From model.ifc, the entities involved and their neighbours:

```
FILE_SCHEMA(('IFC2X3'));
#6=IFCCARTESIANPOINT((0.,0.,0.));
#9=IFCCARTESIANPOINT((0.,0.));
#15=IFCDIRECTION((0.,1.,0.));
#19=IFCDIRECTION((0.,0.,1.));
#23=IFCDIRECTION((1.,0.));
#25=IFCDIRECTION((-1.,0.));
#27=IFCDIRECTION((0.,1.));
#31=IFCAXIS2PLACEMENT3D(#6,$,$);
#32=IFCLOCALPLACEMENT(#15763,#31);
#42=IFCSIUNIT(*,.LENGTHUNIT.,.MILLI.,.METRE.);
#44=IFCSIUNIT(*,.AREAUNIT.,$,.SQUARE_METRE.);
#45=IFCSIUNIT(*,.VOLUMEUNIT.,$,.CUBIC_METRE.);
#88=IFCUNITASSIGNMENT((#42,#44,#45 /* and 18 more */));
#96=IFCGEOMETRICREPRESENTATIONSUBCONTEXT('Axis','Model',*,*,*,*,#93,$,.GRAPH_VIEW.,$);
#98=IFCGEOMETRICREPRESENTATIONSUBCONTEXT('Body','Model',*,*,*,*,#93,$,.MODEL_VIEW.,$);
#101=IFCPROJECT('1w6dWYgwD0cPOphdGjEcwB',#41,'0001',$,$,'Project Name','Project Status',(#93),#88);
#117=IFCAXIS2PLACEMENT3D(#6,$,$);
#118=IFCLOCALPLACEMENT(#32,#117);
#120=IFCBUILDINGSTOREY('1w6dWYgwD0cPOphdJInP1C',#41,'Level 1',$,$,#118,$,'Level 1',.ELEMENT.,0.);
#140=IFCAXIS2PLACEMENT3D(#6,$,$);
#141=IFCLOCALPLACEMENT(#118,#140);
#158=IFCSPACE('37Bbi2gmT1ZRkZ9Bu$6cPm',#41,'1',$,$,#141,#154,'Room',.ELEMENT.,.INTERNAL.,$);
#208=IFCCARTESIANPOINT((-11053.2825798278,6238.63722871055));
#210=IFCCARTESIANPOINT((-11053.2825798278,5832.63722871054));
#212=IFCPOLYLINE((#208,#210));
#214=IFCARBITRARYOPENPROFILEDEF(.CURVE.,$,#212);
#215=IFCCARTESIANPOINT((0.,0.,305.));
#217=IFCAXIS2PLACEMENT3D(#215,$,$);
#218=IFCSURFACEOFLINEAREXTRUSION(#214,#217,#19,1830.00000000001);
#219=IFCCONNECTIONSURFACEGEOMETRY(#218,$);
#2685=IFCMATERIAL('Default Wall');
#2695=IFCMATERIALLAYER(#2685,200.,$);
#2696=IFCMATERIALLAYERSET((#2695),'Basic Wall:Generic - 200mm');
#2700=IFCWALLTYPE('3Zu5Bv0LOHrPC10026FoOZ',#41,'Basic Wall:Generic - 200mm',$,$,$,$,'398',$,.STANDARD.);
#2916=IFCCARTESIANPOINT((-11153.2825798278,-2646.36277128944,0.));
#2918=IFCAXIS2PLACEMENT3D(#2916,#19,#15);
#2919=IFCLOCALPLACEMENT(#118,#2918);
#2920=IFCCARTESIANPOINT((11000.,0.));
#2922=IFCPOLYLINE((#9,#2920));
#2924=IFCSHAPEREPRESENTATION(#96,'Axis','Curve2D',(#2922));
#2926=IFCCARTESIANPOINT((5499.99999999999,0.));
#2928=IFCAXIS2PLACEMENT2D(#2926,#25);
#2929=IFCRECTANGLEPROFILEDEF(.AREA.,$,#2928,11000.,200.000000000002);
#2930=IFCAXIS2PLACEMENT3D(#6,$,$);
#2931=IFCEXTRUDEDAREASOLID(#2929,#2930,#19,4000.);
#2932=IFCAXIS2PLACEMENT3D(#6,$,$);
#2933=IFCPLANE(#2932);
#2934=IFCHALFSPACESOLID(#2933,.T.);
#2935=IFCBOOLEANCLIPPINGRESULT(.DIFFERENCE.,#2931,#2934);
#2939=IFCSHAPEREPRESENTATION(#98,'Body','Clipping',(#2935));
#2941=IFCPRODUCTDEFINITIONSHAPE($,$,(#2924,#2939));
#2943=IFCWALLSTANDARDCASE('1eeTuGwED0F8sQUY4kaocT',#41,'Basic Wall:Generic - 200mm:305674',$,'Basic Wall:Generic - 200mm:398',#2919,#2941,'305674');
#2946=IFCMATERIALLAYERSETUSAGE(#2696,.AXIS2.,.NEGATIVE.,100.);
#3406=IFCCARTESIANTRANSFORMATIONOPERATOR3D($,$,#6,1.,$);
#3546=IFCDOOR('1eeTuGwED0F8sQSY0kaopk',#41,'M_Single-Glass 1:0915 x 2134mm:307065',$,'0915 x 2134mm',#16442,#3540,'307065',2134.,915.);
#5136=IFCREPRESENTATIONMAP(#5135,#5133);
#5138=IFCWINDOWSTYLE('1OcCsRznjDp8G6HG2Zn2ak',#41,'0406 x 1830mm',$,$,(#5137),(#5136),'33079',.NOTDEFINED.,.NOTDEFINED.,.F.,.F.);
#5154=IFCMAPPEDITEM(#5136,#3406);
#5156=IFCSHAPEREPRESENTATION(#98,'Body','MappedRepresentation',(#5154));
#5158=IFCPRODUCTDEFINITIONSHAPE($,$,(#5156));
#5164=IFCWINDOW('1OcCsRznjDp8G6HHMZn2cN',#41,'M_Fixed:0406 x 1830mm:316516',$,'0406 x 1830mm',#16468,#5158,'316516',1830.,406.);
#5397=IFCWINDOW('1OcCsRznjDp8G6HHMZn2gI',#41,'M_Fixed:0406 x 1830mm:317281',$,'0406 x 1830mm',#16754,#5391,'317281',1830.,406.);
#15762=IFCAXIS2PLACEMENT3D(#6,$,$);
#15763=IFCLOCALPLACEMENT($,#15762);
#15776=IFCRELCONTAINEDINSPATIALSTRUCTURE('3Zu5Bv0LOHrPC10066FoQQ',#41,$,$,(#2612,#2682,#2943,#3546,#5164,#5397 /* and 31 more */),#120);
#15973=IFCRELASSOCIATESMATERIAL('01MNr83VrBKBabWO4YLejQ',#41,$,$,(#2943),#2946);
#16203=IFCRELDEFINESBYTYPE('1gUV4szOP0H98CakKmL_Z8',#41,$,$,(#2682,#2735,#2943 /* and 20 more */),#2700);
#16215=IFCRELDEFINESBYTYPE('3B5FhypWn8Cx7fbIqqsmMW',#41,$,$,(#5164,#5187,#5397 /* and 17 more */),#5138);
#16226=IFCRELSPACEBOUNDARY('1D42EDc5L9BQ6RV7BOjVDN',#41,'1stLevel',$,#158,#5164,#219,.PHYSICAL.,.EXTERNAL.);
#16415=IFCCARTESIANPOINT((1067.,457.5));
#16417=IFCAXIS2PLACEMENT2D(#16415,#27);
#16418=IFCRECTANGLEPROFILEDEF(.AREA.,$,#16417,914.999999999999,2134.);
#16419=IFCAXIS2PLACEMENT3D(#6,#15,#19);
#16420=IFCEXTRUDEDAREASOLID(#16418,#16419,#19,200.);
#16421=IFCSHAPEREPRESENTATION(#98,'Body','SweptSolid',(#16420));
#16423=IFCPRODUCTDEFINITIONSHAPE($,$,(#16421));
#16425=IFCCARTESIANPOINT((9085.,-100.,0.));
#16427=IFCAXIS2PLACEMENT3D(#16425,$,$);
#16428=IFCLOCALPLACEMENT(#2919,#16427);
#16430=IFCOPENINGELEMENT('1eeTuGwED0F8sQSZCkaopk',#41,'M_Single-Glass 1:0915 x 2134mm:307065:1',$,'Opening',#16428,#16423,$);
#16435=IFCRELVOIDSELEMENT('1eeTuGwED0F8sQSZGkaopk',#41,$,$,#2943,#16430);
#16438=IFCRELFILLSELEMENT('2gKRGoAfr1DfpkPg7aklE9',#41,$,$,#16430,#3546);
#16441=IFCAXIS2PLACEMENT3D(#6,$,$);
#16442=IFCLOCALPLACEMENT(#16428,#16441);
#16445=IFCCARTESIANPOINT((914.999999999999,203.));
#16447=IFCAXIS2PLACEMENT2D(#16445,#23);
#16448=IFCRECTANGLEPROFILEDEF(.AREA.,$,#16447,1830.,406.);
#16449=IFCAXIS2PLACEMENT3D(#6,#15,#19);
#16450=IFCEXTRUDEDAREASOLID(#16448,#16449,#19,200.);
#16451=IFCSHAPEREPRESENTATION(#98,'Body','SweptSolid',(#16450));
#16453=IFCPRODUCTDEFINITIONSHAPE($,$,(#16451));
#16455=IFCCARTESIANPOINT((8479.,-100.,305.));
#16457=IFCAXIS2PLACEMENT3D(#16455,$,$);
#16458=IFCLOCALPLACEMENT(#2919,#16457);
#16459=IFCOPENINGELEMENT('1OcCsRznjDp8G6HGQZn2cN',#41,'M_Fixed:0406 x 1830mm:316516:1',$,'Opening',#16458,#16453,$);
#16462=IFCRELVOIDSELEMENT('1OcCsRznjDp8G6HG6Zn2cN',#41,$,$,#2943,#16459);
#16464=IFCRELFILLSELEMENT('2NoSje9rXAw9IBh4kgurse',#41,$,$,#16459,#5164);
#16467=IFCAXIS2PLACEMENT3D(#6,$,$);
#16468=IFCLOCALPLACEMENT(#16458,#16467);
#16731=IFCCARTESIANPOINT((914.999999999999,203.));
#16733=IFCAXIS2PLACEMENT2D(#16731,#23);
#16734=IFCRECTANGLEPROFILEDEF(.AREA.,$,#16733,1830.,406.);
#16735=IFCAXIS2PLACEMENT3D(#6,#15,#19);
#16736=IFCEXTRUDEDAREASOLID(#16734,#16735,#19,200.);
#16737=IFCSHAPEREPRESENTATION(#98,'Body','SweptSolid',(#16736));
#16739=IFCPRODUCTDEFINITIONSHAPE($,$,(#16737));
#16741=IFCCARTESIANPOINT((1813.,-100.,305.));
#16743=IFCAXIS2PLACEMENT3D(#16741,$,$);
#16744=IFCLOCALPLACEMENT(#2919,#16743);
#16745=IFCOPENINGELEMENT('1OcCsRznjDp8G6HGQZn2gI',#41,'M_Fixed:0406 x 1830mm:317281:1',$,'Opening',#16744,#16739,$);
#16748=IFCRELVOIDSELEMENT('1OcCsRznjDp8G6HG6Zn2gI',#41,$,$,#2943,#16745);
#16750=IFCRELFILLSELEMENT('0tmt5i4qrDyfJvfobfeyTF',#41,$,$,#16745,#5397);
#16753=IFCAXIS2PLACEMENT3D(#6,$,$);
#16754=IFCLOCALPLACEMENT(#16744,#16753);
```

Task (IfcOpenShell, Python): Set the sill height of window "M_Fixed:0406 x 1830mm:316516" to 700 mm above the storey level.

```python
import numpy as np
import ifcopenshell
import ifcopenshell.api.geometry
import ifcopenshell.geom
import ifcopenshell.util.element
import ifcopenshell.util.placement
import ifcopenshell.util.shape
import ifcopenshell.util.unit

model = ifcopenshell.open("model.ifc")
unit_scale = ifcopenshell.util.unit.calculate_unit_scale(model)

window = model.by_guid("1OcCsRznjDp8G6HHMZn2cN")
opening = window.FillsVoids[0].RelatingOpeningElement
storey = ifcopenshell.util.element.get_container(window, ifc_class="IfcBuildingStorey")
level = ifcopenshell.util.placement.get_local_placement(storey.ObjectPlacement)[2, 3]

# The opening's origin need not be at the sill, so measure its lowest point.
shape = ifcopenshell.geom.create_shape(ifcopenshell.geom.settings(), opening)
bottom = ifcopenshell.util.shape.get_shape_bottom_elevation(shape, shape.geometry) / unit_scale
dz = level + 0.7 / unit_scale - bottom

shift = np.array([0.0, 0.0, dz])
# The window is placed relative to its opening, so it follows when the opening moves.
matrix = ifcopenshell.util.placement.get_local_placement(opening.ObjectPlacement)
matrix[:3, 3] += shift
ifcopenshell.api.geometry.edit_object_placement(
    model, product=opening, matrix=matrix, is_si=False, should_transform_children=True
)

# Space boundary surfaces are stored in each space's coordinates; move them too.
for rel in window.ProvidesBoundaries:
    if not rel.ConnectionGeometry:
        continue
    surface = rel.ConnectionGeometry.SurfaceOnRelatingElement
    space_matrix = ifcopenshell.util.placement.get_local_placement(rel.RelatingSpace.ObjectPlacement)
    point = np.array(surface.Position.Location.Coordinates) + space_matrix[:3, :3].T @ shift
    surface.Position = model.createIfcAxis2Placement3D(
        model.createIfcCartesianPoint(point.tolist()), surface.Position.Axis, surface.Position.RefDirection
    )

print(f"moved by {dz * unit_scale:+.3f} m")

model.write("model_rev.ifc")
```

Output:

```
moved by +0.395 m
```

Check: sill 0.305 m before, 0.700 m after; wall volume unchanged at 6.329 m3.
